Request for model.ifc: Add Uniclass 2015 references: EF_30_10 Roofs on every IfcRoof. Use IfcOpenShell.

First a look at what the model holds.

```python
import ifcopenshell

model = ifcopenshell.open("model.ifc")
print(model.schema)
print("classifications:", [c.Name for c in model.by_type("IfcClassification")])
for ifc_class in ("IfcDoor", "IfcRoof", "IfcStair", "IfcWall", "IfcWindow"):
    print(ifc_class, len(model.by_type(ifc_class)))
```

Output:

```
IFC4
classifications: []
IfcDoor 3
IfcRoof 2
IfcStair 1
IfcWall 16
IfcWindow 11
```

```python
import ifcopenshell
import ifcopenshell.api.classification

model = ifcopenshell.open("model.ifc")

system = ifcopenshell.api.classification.add_classification(model, classification="Uniclass 2015")

codes = {
    "IfcRoof": ("EF_30_10", "Roofs"),
}
for ifc_class, (code, name) in codes.items():
    products = model.by_type(ifc_class)
    ifcopenshell.api.classification.add_reference(
        model, products=products, classification=system, identification=code, name=name
    )
    print(code, len(products))

model.write("model_updated.ifc")
```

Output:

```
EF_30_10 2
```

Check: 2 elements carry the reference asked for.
